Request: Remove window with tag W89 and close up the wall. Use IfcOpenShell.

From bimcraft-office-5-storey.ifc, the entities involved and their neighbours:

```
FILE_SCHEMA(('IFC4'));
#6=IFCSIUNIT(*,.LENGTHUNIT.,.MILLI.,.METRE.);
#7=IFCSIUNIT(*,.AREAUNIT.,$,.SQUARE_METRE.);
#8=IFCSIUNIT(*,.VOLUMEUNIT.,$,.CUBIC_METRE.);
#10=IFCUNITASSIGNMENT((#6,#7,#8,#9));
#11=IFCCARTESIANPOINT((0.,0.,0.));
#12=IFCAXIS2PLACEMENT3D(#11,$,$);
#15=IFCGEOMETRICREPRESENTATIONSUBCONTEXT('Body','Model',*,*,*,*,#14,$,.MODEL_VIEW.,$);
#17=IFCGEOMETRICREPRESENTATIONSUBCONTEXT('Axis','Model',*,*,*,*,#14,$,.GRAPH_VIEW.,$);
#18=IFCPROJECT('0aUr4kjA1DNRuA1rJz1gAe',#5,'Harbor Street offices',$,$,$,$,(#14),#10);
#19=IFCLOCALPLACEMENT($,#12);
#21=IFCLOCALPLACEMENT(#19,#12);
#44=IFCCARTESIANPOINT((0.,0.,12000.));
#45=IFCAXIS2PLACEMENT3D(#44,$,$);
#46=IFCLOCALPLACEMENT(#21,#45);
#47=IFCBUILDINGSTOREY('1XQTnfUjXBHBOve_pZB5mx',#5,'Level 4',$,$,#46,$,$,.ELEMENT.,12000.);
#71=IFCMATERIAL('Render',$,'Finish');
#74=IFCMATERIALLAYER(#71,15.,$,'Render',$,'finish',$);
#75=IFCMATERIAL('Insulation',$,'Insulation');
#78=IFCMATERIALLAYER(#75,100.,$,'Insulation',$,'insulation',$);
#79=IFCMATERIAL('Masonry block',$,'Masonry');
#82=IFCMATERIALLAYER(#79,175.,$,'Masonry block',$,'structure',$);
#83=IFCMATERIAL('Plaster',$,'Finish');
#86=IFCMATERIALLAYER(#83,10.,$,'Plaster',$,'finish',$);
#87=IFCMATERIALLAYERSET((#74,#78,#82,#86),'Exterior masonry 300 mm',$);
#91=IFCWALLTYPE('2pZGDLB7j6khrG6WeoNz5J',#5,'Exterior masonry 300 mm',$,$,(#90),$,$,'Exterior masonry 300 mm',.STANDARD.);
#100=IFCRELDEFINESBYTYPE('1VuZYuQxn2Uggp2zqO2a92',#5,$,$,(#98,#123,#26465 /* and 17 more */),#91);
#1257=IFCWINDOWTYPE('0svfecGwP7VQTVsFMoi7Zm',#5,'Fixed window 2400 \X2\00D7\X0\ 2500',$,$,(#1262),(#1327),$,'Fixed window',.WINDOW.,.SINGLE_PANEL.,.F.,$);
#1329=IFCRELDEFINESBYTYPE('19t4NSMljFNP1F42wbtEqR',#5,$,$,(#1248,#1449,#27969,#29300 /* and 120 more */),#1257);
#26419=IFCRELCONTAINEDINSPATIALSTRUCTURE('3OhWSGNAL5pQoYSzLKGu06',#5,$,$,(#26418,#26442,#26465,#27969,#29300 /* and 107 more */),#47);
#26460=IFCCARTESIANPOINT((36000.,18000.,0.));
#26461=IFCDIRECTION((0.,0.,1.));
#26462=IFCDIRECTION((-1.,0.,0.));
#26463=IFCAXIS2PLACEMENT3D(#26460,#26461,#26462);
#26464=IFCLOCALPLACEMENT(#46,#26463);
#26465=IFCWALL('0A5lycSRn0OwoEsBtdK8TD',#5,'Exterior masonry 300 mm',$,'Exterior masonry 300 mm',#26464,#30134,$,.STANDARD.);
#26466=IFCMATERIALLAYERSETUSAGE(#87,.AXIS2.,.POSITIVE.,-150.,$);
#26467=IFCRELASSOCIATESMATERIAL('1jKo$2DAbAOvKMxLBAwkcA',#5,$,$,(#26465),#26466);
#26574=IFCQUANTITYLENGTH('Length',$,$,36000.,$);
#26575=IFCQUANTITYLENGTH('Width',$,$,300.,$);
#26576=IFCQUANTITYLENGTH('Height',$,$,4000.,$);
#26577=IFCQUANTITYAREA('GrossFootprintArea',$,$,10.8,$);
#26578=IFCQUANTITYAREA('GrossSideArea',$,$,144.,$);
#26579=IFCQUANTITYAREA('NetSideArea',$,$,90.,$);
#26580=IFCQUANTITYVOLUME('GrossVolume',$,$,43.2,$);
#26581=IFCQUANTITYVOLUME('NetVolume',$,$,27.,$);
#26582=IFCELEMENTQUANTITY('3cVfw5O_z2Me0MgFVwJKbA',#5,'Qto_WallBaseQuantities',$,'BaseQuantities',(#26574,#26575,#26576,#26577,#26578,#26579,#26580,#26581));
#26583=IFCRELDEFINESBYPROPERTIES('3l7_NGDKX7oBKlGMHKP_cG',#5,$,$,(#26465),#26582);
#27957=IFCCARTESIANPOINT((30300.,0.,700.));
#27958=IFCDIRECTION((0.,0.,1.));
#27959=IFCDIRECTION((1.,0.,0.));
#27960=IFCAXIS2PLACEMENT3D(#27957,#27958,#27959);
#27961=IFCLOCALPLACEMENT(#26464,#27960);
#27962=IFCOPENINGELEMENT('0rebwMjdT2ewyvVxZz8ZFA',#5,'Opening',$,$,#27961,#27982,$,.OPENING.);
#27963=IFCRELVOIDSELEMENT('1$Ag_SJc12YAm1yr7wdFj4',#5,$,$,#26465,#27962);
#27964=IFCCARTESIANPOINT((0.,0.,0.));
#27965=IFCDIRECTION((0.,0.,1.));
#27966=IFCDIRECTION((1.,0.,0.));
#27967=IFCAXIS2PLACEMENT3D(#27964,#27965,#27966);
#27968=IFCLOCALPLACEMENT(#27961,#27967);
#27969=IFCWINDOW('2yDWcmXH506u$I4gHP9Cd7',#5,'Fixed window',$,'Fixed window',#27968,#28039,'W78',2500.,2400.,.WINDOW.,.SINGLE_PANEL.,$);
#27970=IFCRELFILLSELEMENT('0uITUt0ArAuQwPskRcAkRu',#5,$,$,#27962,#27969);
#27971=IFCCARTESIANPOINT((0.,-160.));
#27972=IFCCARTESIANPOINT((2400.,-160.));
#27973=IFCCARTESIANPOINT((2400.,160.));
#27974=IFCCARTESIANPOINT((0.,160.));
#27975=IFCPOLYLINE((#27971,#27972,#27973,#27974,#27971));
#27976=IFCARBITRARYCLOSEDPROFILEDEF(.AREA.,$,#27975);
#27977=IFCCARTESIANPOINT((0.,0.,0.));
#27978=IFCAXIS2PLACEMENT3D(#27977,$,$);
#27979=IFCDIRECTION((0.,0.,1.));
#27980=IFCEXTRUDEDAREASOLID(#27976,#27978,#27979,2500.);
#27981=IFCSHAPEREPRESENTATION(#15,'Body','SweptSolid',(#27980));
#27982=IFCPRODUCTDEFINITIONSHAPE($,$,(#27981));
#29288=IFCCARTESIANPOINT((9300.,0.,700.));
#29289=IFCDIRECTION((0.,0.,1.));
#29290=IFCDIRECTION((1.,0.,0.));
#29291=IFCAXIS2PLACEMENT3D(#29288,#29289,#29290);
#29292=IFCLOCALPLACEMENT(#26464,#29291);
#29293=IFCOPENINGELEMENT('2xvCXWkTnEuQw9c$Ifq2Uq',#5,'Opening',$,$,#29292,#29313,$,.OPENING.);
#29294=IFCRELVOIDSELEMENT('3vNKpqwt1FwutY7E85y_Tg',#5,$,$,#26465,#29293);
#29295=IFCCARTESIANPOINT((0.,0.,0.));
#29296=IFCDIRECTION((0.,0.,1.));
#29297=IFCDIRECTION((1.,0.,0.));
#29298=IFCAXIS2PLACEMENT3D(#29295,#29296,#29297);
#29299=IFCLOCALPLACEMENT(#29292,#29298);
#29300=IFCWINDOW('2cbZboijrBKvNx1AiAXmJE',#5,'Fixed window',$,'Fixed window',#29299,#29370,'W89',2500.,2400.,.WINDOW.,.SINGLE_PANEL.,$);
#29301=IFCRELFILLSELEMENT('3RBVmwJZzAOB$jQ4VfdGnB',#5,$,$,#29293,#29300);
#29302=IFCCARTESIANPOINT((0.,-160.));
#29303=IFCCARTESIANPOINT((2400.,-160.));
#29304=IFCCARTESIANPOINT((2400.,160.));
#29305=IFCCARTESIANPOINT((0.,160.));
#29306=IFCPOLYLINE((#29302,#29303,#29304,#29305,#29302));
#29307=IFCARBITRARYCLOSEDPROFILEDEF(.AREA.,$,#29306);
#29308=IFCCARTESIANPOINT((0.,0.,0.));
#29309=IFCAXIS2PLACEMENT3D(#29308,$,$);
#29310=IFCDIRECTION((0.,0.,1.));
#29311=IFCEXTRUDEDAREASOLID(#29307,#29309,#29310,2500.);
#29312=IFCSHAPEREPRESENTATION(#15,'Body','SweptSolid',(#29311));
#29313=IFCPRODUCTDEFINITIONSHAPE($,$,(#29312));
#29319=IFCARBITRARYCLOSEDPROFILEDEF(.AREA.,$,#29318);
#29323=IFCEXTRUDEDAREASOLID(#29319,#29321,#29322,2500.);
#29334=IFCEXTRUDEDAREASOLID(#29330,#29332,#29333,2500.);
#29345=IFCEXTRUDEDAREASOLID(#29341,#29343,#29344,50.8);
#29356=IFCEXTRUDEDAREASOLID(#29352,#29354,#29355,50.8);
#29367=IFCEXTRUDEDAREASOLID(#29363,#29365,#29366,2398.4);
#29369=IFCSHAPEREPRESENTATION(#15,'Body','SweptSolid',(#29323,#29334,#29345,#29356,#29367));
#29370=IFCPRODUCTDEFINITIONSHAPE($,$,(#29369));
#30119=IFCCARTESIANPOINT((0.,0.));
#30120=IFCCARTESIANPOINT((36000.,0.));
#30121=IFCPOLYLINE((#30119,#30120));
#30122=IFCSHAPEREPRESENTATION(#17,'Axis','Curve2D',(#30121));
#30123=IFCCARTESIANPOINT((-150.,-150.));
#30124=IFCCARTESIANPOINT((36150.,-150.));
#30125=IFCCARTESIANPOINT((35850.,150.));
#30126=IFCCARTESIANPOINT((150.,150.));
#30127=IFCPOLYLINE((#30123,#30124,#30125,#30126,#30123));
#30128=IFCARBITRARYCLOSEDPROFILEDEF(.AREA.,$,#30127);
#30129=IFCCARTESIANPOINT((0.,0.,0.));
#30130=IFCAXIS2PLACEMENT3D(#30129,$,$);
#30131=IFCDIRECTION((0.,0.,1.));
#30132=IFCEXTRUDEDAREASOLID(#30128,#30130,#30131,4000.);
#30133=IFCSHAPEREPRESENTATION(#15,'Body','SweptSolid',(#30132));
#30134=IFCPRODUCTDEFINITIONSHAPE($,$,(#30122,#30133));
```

```python
import ifcopenshell
import ifcopenshell.api.feature
import ifcopenshell.api.pset
import ifcopenshell.api.root
import ifcopenshell.geom
import ifcopenshell.util.element
import ifcopenshell.util.shape
import ifcopenshell.util.unit

model = ifcopenshell.open("bimcraft-office-5-storey.ifc")
area_scale = ifcopenshell.util.unit.calculate_unit_scale(model, "AREAUNIT")
volume_scale = ifcopenshell.util.unit.calculate_unit_scale(model, "VOLUMEUNIT")
settings = ifcopenshell.geom.settings()


def volume(element):
    """Net volume in cubic metres, openings subtracted."""
    shape = ifcopenshell.geom.create_shape(settings, element)
    return ifcopenshell.util.shape.get_volume(shape.geometry)


window = model.by_id(29300)
opening = window.FillsVoids[0].RelatingOpeningElement
wall = opening.VoidsElements[0].RelatingBuildingElement
before = volume(wall)

ifcopenshell.api.root.remove_product(model, product=window)
ifcopenshell.api.feature.remove_feature(model, feature=opening)

after = volume(wall)
thickness = 0.3  # wall thickness in metres

# Update the wall's stored quantities.
qto = model.by_id(ifcopenshell.util.element.get_pset(wall, "Qto_WallBaseQuantities", should_inherit=False)["id"])
ifcopenshell.api.pset.edit_qto(model, qto=qto, properties={
    "NetSideArea": after / thickness / area_scale,
    "NetVolume": after / volume_scale,
})

print(f"wall volume {before:.3f} -> {after:.3f} m3")

model.write("bimcraft-office-5-storey_v2.ifc")
```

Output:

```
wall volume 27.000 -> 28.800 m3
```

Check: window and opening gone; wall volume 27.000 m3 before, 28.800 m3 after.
